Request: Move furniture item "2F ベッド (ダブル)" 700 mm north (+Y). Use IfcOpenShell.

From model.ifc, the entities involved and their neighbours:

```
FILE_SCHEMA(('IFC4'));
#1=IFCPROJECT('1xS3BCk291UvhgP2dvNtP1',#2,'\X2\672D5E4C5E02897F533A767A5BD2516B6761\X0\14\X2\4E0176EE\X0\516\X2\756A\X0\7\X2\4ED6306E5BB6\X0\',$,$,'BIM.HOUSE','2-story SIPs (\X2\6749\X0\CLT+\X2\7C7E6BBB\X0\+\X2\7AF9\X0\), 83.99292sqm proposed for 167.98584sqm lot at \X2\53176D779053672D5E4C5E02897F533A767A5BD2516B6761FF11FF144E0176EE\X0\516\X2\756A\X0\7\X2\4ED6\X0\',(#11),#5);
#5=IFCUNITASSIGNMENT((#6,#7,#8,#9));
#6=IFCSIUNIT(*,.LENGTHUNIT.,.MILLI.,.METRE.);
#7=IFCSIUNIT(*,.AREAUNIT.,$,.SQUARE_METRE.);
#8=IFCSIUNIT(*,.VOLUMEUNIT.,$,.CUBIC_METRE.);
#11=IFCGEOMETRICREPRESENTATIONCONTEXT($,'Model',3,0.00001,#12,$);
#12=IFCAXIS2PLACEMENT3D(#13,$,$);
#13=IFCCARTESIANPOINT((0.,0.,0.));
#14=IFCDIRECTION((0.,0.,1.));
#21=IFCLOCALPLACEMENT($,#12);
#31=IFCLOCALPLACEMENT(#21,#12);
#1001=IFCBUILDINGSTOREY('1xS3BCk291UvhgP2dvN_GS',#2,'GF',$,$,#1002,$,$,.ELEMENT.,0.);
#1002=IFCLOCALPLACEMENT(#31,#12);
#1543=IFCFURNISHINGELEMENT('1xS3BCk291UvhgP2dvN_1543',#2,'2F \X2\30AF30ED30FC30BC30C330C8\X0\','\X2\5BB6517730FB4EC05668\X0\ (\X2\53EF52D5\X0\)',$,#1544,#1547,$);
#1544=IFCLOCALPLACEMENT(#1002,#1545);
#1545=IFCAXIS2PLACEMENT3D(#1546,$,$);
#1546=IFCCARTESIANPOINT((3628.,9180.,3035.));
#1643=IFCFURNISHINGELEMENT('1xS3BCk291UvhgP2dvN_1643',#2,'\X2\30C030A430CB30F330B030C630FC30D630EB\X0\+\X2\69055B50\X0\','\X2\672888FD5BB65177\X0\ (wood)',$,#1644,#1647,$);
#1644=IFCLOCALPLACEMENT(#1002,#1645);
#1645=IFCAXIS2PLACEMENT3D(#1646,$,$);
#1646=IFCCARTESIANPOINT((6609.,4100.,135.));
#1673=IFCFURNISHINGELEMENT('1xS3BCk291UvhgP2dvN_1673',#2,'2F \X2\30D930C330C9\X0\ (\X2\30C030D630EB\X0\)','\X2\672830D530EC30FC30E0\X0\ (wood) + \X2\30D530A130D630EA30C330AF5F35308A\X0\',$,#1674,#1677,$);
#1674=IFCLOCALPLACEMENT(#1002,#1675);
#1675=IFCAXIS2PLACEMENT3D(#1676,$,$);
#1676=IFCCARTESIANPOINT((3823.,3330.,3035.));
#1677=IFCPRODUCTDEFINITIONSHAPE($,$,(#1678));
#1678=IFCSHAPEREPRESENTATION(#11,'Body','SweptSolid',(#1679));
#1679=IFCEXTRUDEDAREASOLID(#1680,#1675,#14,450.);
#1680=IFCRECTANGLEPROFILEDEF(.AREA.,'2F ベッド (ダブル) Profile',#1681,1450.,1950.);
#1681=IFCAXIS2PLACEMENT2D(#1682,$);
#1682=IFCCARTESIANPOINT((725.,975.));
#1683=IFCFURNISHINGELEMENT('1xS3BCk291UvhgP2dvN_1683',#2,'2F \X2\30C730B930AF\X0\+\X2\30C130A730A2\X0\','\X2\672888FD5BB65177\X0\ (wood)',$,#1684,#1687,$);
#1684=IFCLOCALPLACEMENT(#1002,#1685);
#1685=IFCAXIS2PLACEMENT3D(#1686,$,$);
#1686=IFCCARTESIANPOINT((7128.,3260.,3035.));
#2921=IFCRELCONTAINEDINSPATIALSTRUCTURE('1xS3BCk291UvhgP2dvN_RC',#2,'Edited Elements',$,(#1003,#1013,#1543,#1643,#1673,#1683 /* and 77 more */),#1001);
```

```python
import ifcopenshell
import ifcopenshell.api.geometry
import ifcopenshell.util.placement

model = ifcopenshell.open("model.ifc")

item = model.by_id(1673)
matrix = ifcopenshell.util.placement.get_local_placement(item.ObjectPlacement)
matrix[1, 3] += 700.0
ifcopenshell.api.geometry.edit_object_placement(model, product=item, matrix=matrix, is_si=False)

print(ifcopenshell.util.placement.get_local_placement(item.ObjectPlacement).round(3) + 0.0)

model.write("model_v2.ifc")
```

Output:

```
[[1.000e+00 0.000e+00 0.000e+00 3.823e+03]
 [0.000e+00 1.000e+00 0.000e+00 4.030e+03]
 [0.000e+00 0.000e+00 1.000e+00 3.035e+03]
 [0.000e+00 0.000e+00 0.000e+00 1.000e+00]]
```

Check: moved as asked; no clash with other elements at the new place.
